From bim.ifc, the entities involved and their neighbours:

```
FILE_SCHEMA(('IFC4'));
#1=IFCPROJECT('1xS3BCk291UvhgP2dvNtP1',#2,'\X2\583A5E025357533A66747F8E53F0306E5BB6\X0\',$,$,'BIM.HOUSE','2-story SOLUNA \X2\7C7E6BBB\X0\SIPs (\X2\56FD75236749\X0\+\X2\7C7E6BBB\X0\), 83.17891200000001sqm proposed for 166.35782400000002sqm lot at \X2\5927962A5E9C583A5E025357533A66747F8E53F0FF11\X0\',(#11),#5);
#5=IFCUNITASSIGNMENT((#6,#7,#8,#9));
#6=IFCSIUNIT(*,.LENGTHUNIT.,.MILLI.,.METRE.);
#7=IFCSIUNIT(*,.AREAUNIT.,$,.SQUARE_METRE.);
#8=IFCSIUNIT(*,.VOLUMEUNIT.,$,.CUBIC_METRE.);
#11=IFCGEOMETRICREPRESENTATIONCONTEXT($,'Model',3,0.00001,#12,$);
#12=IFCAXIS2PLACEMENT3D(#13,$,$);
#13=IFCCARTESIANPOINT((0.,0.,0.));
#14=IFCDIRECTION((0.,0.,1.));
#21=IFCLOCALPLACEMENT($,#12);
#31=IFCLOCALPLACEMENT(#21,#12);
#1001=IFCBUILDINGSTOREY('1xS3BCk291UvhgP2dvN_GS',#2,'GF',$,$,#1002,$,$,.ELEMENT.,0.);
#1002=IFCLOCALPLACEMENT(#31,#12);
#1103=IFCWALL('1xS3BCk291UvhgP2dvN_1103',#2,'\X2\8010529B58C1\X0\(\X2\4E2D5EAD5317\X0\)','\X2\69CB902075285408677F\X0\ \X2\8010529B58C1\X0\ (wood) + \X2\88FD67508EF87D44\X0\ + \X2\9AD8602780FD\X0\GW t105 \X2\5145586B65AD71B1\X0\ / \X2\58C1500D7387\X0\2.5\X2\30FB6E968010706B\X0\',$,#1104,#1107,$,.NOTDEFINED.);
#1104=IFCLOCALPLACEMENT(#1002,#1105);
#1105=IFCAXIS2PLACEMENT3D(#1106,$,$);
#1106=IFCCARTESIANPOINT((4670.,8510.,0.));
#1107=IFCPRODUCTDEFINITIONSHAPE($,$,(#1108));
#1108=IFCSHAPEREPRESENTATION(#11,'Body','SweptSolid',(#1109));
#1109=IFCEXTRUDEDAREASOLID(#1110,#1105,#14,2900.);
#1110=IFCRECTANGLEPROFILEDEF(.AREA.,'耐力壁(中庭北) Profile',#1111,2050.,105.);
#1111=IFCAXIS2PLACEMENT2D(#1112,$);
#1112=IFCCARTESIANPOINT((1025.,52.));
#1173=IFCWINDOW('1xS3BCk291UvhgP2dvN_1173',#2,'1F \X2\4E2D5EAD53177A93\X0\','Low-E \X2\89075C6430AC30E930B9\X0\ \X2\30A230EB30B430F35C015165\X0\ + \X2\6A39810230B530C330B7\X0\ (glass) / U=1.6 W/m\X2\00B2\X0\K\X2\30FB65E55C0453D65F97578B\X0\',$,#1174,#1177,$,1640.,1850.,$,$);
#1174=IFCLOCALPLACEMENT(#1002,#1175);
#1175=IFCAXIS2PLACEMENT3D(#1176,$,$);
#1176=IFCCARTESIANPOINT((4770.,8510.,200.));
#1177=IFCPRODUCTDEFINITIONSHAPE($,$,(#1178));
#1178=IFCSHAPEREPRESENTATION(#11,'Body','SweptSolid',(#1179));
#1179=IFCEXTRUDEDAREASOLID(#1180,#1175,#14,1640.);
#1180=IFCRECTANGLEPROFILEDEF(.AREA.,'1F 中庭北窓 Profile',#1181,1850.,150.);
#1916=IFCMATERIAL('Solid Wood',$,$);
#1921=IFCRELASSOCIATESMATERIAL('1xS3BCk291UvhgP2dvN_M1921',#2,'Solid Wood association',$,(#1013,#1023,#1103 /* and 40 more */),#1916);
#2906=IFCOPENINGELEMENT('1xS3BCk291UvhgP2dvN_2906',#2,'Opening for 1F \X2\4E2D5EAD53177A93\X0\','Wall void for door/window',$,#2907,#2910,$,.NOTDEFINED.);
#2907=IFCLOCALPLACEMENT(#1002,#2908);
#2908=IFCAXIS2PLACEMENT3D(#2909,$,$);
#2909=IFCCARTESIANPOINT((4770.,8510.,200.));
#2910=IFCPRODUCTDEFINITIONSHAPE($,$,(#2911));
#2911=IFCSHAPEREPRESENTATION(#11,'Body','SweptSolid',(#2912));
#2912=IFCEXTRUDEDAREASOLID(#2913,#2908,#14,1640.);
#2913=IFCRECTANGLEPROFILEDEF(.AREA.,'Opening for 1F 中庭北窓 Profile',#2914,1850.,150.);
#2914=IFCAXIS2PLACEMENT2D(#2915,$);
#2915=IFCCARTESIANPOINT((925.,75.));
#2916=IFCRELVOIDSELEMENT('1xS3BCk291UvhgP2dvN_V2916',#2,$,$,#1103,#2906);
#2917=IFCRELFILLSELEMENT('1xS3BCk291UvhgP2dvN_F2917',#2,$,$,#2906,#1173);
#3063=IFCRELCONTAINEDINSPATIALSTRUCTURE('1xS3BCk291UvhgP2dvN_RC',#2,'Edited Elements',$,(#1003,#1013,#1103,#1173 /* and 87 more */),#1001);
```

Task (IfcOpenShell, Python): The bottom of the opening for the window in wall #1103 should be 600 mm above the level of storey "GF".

```python
import numpy as np
import ifcopenshell
import ifcopenshell.api.geometry
import ifcopenshell.geom
import ifcopenshell.util.element
import ifcopenshell.util.placement
import ifcopenshell.util.shape
import ifcopenshell.util.unit

model = ifcopenshell.open("bim.ifc")
unit_scale = ifcopenshell.util.unit.calculate_unit_scale(model)

window = model.by_guid("1xS3BCk291UvhgP2dvN_1173")
opening = window.FillsVoids[0].RelatingOpeningElement
storey = ifcopenshell.util.element.get_container(window, ifc_class="IfcBuildingStorey")
level = ifcopenshell.util.placement.get_local_placement(storey.ObjectPlacement)[2, 3]

# The opening's origin need not be at the sill, so measure its lowest point.
shape = ifcopenshell.geom.create_shape(ifcopenshell.geom.settings(), opening)
bottom = ifcopenshell.util.shape.get_shape_bottom_elevation(shape, shape.geometry) / unit_scale
dz = level + 600.0 - bottom

shift = np.array([0.0, 0.0, dz])
# The window is not placed relative to its opening, so move both.
for product in (opening, window):
    matrix = ifcopenshell.util.placement.get_local_placement(product.ObjectPlacement)
    matrix[:3, 3] += shift
    ifcopenshell.api.geometry.edit_object_placement(model, product=product, matrix=matrix, is_si=False)

print(f"moved by {dz * unit_scale:+.3f} m")

model.write("bim_updated.ifc")
```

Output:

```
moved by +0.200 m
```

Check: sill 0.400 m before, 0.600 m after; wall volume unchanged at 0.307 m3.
